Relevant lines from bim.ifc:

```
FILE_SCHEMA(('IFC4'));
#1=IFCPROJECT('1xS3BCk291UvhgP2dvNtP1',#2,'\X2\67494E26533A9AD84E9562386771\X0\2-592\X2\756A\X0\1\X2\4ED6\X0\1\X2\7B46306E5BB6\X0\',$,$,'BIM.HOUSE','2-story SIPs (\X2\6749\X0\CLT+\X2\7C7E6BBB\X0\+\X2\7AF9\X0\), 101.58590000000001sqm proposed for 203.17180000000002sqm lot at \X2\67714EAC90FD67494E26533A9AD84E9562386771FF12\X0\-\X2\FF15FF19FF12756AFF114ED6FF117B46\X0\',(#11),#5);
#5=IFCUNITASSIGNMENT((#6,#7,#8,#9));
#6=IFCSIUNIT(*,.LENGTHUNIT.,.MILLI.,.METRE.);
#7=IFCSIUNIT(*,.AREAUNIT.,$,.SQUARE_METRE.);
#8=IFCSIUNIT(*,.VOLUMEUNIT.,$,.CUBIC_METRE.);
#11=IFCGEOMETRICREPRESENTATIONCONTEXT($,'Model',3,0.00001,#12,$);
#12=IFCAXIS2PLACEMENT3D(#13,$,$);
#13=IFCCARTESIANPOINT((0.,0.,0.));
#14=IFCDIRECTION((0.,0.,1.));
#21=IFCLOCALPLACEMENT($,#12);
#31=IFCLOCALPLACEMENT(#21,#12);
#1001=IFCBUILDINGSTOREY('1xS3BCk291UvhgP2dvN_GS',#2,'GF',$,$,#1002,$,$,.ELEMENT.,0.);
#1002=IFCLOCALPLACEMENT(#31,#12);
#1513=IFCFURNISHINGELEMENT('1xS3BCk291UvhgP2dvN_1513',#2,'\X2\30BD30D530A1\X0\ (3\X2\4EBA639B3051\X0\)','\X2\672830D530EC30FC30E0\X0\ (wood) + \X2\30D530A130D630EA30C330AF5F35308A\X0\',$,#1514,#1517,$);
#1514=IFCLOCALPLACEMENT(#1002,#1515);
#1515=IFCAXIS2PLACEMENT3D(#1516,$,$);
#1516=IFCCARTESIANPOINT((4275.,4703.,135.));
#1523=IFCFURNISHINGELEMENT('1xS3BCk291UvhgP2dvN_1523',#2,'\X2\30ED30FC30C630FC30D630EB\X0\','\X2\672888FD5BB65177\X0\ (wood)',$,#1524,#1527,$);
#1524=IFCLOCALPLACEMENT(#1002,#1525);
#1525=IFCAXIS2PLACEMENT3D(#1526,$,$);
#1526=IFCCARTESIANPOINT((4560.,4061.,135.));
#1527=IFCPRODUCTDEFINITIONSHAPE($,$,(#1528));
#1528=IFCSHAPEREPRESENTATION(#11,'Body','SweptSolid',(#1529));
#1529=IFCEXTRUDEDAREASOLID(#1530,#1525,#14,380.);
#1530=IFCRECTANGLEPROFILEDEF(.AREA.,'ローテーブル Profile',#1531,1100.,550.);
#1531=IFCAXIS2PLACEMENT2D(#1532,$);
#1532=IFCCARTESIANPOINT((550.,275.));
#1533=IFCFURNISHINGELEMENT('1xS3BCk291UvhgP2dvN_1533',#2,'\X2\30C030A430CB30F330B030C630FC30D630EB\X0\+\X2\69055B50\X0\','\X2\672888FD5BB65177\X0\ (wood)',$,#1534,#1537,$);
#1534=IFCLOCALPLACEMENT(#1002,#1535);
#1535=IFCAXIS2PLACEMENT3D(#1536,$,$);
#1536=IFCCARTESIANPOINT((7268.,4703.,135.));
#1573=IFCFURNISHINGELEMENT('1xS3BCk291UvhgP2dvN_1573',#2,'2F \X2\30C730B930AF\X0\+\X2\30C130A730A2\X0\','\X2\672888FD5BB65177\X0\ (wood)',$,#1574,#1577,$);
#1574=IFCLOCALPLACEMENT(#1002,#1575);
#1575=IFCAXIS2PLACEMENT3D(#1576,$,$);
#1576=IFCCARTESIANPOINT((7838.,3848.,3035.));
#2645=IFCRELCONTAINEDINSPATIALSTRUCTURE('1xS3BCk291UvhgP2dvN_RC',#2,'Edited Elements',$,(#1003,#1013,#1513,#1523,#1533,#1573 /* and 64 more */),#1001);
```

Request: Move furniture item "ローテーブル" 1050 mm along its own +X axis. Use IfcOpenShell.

```python
import ifcopenshell
import ifcopenshell.api.geometry
import ifcopenshell.util.placement
import ifcopenshell.util.unit

model = ifcopenshell.open("bim.ifc")
unit_scale = ifcopenshell.util.unit.calculate_unit_scale(model)

item = model.by_guid("1xS3BCk291UvhgP2dvN_1523")
matrix = ifcopenshell.util.placement.get_local_placement(item.ObjectPlacement)
matrix[:3, 3] += matrix[:3, 0] * 1.05 / unit_scale
ifcopenshell.api.geometry.edit_object_placement(model, product=item, matrix=matrix, is_si=False)

print(ifcopenshell.util.placement.get_local_placement(item.ObjectPlacement).round(3) + 0.0)

model.write("bim_v2.ifc")
```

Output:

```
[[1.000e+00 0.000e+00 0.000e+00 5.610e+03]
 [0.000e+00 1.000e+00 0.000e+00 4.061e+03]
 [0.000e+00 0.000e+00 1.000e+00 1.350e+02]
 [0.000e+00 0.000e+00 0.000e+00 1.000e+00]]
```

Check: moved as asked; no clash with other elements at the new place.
